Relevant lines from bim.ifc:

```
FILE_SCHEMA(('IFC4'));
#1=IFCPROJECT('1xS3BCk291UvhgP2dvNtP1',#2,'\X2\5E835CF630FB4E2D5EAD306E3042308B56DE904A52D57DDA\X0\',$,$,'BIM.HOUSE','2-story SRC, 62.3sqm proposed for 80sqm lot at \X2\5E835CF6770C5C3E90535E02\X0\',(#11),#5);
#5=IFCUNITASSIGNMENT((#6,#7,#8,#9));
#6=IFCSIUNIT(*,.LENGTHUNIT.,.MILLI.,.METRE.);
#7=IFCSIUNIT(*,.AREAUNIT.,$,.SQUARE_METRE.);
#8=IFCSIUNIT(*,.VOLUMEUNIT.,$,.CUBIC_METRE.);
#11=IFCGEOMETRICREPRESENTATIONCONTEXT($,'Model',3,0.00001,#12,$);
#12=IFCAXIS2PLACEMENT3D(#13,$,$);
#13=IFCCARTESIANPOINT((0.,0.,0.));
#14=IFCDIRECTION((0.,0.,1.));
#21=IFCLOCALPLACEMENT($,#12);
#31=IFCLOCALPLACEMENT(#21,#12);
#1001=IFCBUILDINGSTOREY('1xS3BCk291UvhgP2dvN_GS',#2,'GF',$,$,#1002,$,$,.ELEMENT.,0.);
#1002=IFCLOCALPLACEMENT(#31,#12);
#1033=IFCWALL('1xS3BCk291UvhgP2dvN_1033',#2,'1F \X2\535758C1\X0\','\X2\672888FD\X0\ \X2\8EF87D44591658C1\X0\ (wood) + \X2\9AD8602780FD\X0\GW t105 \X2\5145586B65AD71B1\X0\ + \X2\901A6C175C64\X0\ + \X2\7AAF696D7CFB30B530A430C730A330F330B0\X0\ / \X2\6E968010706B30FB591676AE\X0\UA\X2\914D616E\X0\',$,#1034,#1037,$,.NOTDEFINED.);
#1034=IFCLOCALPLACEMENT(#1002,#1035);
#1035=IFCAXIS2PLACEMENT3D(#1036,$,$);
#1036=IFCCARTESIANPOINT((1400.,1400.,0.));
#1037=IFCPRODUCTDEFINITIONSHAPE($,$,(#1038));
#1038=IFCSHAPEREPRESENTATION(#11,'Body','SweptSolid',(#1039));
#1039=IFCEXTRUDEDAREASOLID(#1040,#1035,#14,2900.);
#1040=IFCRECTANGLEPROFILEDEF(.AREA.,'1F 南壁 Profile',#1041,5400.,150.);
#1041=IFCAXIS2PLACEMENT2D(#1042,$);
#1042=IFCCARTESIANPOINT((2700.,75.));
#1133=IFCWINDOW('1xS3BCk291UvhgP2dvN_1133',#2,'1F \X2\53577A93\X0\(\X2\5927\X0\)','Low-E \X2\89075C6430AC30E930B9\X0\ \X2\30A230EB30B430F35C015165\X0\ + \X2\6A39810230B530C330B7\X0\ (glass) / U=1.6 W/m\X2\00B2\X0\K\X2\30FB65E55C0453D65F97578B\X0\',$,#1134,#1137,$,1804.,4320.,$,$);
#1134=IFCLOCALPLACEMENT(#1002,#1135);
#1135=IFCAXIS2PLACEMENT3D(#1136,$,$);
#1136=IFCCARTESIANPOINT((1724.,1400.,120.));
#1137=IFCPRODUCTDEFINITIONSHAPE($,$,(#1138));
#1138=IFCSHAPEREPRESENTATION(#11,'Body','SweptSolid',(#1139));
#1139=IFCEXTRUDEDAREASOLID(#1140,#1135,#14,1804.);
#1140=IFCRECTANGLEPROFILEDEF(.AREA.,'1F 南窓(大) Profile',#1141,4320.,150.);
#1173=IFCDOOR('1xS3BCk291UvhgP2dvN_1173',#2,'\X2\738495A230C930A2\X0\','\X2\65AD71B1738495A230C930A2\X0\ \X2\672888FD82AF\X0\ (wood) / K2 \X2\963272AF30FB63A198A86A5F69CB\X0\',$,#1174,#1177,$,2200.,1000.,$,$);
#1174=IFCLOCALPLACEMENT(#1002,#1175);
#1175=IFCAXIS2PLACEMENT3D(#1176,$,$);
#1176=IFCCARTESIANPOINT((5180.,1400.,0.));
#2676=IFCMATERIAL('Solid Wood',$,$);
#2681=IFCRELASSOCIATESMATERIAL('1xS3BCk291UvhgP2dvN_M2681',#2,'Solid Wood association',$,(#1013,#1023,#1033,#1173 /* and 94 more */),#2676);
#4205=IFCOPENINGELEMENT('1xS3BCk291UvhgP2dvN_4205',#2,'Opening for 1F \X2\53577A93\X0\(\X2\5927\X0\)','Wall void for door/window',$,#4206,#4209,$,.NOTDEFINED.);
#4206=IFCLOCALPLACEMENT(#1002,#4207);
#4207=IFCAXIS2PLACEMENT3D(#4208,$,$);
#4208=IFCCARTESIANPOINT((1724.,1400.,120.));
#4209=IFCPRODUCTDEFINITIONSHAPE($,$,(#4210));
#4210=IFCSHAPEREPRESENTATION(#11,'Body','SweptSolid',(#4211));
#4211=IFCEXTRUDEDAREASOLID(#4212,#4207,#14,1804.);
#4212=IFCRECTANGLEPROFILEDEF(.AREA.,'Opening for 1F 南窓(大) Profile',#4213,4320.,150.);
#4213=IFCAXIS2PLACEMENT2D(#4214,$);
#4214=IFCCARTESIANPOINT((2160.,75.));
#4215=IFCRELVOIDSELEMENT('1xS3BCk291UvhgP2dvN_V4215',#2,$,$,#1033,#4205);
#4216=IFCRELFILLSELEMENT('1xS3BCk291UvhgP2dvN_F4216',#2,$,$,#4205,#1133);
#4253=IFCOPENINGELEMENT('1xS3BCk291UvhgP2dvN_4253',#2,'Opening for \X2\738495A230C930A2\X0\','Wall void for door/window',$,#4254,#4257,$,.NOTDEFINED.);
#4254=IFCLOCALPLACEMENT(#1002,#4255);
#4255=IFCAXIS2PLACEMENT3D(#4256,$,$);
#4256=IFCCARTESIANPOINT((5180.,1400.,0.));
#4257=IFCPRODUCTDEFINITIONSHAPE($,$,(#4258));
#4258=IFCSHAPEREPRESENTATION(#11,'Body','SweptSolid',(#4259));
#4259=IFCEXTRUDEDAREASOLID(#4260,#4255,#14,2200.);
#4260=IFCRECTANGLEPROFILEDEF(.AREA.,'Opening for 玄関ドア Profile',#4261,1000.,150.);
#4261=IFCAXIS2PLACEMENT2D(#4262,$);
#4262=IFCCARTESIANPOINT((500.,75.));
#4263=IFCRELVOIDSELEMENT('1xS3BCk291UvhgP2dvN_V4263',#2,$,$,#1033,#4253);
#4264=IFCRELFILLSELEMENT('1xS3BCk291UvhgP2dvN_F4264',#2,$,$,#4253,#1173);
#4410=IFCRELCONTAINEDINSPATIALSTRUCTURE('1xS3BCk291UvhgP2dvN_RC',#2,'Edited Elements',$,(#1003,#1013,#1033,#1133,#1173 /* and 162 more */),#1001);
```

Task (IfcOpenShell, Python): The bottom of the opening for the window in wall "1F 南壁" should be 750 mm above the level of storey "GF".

```python
import numpy as np
import ifcopenshell
import ifcopenshell.api.geometry
import ifcopenshell.geom
import ifcopenshell.util.element
import ifcopenshell.util.placement
import ifcopenshell.util.shape
import ifcopenshell.util.unit

model = ifcopenshell.open("bim.ifc")
unit_scale = ifcopenshell.util.unit.calculate_unit_scale(model)

window = model.by_guid("1xS3BCk291UvhgP2dvN_1133")
opening = window.FillsVoids[0].RelatingOpeningElement
storey = ifcopenshell.util.element.get_container(window, ifc_class="IfcBuildingStorey")
level = ifcopenshell.util.placement.get_local_placement(storey.ObjectPlacement)[2, 3]

# The opening's origin need not be at the sill, so measure its lowest point.
shape = ifcopenshell.geom.create_shape(ifcopenshell.geom.settings(), opening)
bottom = ifcopenshell.util.shape.get_shape_bottom_elevation(shape, shape.geometry) / unit_scale
dz = level + 750.0 - bottom

shift = np.array([0.0, 0.0, dz])
# The window is not placed relative to its opening, so move both.
for product in (opening, window):
    matrix = ifcopenshell.util.placement.get_local_placement(product.ObjectPlacement)
    matrix[:3, 3] += shift
    ifcopenshell.api.geometry.edit_object_placement(model, product=product, matrix=matrix, is_si=False)

print(f"moved by {dz * unit_scale:+.3f} m")

model.write("bim-out.ifc")
```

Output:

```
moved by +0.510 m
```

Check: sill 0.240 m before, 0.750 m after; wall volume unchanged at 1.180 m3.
